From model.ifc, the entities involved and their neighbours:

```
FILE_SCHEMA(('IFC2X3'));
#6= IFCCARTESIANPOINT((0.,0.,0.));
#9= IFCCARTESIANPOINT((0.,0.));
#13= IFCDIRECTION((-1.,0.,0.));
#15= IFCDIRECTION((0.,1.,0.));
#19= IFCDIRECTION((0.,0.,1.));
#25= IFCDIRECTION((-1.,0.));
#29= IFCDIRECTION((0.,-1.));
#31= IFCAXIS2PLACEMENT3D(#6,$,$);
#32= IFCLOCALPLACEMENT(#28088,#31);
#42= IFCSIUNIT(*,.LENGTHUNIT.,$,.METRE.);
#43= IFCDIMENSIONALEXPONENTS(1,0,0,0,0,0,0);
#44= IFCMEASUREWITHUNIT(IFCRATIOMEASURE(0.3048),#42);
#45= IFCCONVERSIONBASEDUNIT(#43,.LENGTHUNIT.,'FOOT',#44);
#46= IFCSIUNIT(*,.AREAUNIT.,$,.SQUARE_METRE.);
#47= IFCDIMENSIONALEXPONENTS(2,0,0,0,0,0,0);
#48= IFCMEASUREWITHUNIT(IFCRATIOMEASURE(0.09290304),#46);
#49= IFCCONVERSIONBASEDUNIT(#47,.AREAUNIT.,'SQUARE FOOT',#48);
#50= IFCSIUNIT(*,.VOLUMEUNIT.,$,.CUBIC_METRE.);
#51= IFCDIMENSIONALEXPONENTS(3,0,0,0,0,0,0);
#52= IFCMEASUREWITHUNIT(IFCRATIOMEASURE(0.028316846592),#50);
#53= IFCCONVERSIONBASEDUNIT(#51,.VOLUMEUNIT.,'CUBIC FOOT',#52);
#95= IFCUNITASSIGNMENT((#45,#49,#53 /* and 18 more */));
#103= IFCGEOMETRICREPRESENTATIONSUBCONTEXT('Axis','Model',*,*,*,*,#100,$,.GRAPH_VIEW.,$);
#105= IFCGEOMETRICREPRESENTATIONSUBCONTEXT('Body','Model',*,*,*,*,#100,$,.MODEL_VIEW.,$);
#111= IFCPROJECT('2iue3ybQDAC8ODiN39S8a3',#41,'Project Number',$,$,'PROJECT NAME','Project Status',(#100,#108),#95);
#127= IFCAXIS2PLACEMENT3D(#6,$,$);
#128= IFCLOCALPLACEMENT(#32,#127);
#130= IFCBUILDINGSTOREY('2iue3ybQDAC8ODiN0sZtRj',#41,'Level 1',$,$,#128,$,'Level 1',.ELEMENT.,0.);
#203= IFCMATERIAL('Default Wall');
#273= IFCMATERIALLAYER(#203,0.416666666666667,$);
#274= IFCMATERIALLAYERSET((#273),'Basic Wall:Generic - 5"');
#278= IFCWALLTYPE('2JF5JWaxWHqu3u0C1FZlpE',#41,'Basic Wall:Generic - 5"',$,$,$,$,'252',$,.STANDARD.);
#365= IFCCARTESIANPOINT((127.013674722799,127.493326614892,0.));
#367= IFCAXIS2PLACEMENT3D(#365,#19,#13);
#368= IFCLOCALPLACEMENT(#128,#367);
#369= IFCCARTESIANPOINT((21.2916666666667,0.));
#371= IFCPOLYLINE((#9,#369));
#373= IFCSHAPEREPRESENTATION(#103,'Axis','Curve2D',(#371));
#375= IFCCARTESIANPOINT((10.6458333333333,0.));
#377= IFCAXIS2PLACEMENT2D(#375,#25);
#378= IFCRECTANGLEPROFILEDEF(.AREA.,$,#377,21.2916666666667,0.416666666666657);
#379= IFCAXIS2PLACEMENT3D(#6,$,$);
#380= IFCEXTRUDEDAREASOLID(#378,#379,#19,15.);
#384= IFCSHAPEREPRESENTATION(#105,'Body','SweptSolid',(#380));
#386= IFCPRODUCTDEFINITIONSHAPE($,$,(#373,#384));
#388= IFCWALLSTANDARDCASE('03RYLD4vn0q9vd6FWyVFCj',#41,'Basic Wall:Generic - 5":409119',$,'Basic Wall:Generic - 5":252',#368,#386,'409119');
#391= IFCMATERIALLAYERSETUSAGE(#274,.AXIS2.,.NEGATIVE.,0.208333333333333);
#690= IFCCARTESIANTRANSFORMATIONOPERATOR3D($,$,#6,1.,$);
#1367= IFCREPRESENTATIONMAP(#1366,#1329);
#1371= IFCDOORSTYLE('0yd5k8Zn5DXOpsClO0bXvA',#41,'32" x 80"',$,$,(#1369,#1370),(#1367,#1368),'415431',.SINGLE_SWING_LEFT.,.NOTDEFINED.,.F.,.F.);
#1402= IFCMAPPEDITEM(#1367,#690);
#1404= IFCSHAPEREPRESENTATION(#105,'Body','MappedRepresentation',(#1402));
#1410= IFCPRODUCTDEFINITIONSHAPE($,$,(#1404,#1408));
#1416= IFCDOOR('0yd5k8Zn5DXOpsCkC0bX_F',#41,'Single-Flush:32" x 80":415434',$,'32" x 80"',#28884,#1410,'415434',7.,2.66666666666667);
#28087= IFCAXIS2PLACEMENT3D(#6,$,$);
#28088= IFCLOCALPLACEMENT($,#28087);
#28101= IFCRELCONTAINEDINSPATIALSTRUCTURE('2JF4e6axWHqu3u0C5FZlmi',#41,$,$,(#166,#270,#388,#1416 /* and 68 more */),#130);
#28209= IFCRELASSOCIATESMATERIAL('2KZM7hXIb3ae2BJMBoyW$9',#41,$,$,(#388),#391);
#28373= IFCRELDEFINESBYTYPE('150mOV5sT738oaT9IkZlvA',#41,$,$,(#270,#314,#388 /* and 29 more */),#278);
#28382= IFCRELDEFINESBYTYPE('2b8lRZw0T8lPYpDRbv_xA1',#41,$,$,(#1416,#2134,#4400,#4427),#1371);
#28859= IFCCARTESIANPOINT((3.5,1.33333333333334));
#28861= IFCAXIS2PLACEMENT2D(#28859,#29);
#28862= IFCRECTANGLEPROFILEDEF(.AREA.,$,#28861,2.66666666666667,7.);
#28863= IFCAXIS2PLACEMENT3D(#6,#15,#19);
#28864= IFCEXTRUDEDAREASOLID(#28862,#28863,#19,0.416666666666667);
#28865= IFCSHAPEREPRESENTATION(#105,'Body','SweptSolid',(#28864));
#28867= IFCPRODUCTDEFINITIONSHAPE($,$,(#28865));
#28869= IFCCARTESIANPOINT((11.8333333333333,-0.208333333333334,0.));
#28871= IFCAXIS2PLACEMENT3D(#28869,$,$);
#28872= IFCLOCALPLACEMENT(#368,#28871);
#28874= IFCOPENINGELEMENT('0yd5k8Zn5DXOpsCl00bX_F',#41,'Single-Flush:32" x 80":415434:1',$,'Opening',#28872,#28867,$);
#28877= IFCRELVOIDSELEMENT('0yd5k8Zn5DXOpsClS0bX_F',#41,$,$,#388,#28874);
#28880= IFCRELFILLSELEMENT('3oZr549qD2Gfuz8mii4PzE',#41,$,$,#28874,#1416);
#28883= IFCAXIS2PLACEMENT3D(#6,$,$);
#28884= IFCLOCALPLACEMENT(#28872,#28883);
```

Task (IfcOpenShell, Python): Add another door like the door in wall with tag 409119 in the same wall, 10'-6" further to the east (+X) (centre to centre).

```python
import ifcopenshell
import ifcopenshell.api.feature
import ifcopenshell.api.geometry
import ifcopenshell.api.root
import ifcopenshell.geom
import ifcopenshell.util.element
import ifcopenshell.util.placement
import ifcopenshell.util.shape
import ifcopenshell.util.unit

model = ifcopenshell.open("model.ifc")
unit_scale = ifcopenshell.util.unit.calculate_unit_scale(model)
settings = ifcopenshell.geom.settings()


def volume(element):
    """Net volume in cubic metres, openings subtracted."""
    shape = ifcopenshell.geom.create_shape(settings, element)
    return ifcopenshell.util.shape.get_volume(shape.geometry)


def reuse_history(source, copy):
    """copy_class also copies each property set's owner history, people and application; keep the originals."""
    for rel in copy.IsDefinedBy:
        if rel.is_a("IfcRelDefinesByProperties") and (history := rel.RelatingPropertyDefinition.OwnerHistory):
            rel.RelatingPropertyDefinition.OwnerHistory = source.OwnerHistory
            ifcopenshell.util.element.remove_deep2(model, history)


door = model.by_guid("0yd5k8Zn5DXOpsCkC0bX_F")
opening = door.FillsVoids[0].RelatingOpeningElement
wall = opening.VoidsElements[0].RelatingBuildingElement
before = volume(wall)
shift = ifcopenshell.util.placement.get_local_placement(wall.ObjectPlacement)[:3, 0] * -126 * 0.0254 / unit_scale

# copy_class copies the void relationship, type, container and properties, but no geometry.
new_opening = ifcopenshell.api.root.copy_class(model, product=opening)
new_opening.Representation = ifcopenshell.util.element.copy_deep(
    model, opening.Representation, exclude=["IfcGeometricRepresentationContext", "IfcRepresentationMap"]
)
new_opening.Name = 'Single-Flush:32" x 80"'
new_door = ifcopenshell.api.root.copy_class(model, product=door)
new_door.Representation = ifcopenshell.util.element.copy_deep(
    model, door.Representation, exclude=["IfcGeometricRepresentationContext", "IfcRepresentationMap"]
)
new_door.Name = 'Single-Flush:32" x 80"'
new_door.Tag = None
reuse_history(door, new_door)
fills = ifcopenshell.api.feature.add_filling(model, opening=new_opening, element=new_door)
fills.OwnerHistory = new_door.OwnerHistory  # required in IFC2X3

for old, new in ((opening, new_opening), (door, new_door)):
    matrix = ifcopenshell.util.placement.get_local_placement(old.ObjectPlacement)
    matrix[:3, 3] += shift
    ifcopenshell.api.geometry.edit_object_placement(model, product=new, matrix=matrix, is_si=False)

after = volume(wall)

print(f"wall volume {before:.3f} -> {after:.3f} m3")

model.write("model_updated.ifc")
```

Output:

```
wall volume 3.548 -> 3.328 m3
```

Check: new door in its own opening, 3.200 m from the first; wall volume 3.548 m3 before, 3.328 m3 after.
